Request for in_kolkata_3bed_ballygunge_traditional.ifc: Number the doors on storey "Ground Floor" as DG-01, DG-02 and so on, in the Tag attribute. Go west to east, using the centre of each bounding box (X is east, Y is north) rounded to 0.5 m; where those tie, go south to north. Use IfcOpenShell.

First a look at what the model holds.

```python
import ifcopenshell
import ifcopenshell.util.element
import ifcopenshell.util.placement

model = ifcopenshell.open("in_kolkata_3bed_ballygunge_traditional.ifc")
print(model.schema)
storey = next(s for s in model.by_type("IfcBuildingStorey") if s.Name == "Ground Floor")
doors = [e for e in ifcopenshell.util.element.get_decomposition(storey) if e.is_a("IfcDoor")]
for e in sorted(doors, key=lambda e: e.id()):
    origin = ifcopenshell.util.placement.get_local_placement(e.ObjectPlacement)[:3, 3]
    print(e.id(), e.Tag, e.Name, origin.round(2) + 0.0, sep=" | ")
```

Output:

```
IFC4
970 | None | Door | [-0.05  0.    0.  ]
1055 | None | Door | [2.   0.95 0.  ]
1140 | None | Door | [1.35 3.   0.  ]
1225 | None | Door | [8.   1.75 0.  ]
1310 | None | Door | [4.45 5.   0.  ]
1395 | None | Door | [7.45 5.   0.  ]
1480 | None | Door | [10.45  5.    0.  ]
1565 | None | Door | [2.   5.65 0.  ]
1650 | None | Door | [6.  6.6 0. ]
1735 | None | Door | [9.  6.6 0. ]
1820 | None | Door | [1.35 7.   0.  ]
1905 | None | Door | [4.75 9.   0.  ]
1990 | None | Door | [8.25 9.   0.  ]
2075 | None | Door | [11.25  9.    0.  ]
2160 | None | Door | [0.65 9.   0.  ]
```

```python
import ifcopenshell
import ifcopenshell.geom
import ifcopenshell.util.element
import ifcopenshell.util.shape

model = ifcopenshell.open("in_kolkata_3bed_ballygunge_traditional.ifc")
settings = ifcopenshell.geom.settings()
settings.set("use-world-coords", True)


def centre(element):
    shape = ifcopenshell.geom.create_shape(settings, element)
    return ifcopenshell.util.shape.get_bbox_centroid(shape.geometry)


storey = next(s for s in model.by_type("IfcBuildingStorey") if s.Name == "Ground Floor")
doors = [e for e in ifcopenshell.util.element.get_decomposition(storey) if e.is_a("IfcDoor")]

# Insertion points can sit at a corner or the storey origin, so sort by the geometry (in metres).
centres = {e: centre(e) for e in doors}
doors.sort(key=lambda e: (round(centres[e][0] / 0.5), centres[e][1]))

for i, e in enumerate(doors, start=1):
    number = f"DG-{i:02d}"
    e.Tag = number
    print(e.id(), number)

model.write("in_kolkata_3bed_ballygunge_traditional-out.ifc")
```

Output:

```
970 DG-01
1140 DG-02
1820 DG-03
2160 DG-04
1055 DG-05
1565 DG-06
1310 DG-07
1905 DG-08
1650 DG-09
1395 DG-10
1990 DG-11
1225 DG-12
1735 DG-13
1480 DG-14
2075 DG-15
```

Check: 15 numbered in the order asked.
